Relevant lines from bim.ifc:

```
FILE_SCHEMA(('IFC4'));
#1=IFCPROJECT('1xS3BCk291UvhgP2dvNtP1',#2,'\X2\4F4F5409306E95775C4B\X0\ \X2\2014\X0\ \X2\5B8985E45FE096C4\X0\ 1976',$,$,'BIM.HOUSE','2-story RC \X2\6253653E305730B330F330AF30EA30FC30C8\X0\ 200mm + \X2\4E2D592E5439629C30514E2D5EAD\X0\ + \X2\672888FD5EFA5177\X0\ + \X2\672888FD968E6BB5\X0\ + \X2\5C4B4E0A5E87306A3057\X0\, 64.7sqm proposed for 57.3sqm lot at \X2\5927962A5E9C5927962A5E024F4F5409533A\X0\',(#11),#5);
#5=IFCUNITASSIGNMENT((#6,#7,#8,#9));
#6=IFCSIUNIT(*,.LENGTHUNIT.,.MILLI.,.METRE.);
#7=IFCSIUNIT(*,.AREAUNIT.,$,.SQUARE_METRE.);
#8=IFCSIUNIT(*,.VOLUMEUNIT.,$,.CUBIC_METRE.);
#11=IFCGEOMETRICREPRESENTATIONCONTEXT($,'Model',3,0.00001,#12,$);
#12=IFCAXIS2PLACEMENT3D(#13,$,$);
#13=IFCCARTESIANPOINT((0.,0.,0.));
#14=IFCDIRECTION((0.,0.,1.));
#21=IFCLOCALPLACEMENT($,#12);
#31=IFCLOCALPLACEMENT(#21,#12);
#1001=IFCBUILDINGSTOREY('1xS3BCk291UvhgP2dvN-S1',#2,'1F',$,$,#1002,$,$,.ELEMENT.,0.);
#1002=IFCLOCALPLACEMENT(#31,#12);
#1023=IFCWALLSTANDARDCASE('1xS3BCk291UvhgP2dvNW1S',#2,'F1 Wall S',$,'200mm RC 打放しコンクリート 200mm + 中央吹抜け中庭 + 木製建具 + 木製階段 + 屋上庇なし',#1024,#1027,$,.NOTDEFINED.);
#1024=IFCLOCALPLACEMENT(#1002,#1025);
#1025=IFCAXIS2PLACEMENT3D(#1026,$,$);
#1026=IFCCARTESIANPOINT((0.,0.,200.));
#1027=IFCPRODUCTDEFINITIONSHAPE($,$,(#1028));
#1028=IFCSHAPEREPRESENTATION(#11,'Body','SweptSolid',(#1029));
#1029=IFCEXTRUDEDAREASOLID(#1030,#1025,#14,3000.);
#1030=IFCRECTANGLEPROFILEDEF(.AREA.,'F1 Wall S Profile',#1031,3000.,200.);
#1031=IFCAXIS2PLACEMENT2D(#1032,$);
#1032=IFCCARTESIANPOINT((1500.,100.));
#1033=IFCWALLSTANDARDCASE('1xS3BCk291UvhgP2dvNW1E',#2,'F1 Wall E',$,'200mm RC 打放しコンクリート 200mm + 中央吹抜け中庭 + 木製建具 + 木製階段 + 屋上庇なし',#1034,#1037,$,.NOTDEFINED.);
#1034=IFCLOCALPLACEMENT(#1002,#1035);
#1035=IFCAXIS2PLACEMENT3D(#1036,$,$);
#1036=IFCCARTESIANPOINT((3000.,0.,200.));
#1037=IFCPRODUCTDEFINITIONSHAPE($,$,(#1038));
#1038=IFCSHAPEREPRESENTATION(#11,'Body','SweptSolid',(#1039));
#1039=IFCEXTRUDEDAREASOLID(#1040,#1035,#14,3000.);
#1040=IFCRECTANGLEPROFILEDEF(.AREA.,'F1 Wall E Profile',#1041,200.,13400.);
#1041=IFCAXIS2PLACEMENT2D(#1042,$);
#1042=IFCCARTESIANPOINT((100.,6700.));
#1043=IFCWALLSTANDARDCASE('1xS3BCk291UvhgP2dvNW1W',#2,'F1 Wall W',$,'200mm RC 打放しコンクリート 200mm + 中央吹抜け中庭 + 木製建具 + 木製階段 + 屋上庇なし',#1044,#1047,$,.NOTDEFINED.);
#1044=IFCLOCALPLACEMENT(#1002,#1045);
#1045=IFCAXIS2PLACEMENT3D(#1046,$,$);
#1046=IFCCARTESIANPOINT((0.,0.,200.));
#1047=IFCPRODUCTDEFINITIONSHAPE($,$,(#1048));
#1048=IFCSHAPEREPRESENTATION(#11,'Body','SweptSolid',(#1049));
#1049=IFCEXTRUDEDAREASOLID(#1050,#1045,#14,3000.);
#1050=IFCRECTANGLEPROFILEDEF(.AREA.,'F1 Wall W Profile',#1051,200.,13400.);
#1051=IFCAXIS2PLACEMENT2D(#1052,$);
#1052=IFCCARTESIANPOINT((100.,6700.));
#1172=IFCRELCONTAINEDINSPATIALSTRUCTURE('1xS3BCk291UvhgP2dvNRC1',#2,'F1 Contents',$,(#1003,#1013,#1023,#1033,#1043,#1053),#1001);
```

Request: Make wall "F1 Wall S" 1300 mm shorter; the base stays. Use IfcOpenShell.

```python
import ifcopenshell
import ifcopenshell.geom
import ifcopenshell.util.shape
import ifcopenshell.util.unit

model = ifcopenshell.open("bim.ifc")
unit_scale = ifcopenshell.util.unit.calculate_unit_scale(model)
settings = ifcopenshell.geom.settings()


def volume(element):
    """Net volume in cubic metres, openings subtracted."""
    shape = ifcopenshell.geom.create_shape(settings, element)
    return ifcopenshell.util.shape.get_volume(shape.geometry)


wall = model.by_guid("1xS3BCk291UvhgP2dvNW1S")
before = volume(wall)

body = next(r for r in wall.Representation.Representations if r.RepresentationIdentifier == "Body")
solid = body.Items[0]
old_height = solid.Depth
solid.Depth -= 1.3 / unit_scale
after = volume(wall)

print(f"height {old_height:g} -> {solid.Depth:g}, volume {before:.3f} -> {after:.3f} m3")

model.write("bim_v2.ifc")
```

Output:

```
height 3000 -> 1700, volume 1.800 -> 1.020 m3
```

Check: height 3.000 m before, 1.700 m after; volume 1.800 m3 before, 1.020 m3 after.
